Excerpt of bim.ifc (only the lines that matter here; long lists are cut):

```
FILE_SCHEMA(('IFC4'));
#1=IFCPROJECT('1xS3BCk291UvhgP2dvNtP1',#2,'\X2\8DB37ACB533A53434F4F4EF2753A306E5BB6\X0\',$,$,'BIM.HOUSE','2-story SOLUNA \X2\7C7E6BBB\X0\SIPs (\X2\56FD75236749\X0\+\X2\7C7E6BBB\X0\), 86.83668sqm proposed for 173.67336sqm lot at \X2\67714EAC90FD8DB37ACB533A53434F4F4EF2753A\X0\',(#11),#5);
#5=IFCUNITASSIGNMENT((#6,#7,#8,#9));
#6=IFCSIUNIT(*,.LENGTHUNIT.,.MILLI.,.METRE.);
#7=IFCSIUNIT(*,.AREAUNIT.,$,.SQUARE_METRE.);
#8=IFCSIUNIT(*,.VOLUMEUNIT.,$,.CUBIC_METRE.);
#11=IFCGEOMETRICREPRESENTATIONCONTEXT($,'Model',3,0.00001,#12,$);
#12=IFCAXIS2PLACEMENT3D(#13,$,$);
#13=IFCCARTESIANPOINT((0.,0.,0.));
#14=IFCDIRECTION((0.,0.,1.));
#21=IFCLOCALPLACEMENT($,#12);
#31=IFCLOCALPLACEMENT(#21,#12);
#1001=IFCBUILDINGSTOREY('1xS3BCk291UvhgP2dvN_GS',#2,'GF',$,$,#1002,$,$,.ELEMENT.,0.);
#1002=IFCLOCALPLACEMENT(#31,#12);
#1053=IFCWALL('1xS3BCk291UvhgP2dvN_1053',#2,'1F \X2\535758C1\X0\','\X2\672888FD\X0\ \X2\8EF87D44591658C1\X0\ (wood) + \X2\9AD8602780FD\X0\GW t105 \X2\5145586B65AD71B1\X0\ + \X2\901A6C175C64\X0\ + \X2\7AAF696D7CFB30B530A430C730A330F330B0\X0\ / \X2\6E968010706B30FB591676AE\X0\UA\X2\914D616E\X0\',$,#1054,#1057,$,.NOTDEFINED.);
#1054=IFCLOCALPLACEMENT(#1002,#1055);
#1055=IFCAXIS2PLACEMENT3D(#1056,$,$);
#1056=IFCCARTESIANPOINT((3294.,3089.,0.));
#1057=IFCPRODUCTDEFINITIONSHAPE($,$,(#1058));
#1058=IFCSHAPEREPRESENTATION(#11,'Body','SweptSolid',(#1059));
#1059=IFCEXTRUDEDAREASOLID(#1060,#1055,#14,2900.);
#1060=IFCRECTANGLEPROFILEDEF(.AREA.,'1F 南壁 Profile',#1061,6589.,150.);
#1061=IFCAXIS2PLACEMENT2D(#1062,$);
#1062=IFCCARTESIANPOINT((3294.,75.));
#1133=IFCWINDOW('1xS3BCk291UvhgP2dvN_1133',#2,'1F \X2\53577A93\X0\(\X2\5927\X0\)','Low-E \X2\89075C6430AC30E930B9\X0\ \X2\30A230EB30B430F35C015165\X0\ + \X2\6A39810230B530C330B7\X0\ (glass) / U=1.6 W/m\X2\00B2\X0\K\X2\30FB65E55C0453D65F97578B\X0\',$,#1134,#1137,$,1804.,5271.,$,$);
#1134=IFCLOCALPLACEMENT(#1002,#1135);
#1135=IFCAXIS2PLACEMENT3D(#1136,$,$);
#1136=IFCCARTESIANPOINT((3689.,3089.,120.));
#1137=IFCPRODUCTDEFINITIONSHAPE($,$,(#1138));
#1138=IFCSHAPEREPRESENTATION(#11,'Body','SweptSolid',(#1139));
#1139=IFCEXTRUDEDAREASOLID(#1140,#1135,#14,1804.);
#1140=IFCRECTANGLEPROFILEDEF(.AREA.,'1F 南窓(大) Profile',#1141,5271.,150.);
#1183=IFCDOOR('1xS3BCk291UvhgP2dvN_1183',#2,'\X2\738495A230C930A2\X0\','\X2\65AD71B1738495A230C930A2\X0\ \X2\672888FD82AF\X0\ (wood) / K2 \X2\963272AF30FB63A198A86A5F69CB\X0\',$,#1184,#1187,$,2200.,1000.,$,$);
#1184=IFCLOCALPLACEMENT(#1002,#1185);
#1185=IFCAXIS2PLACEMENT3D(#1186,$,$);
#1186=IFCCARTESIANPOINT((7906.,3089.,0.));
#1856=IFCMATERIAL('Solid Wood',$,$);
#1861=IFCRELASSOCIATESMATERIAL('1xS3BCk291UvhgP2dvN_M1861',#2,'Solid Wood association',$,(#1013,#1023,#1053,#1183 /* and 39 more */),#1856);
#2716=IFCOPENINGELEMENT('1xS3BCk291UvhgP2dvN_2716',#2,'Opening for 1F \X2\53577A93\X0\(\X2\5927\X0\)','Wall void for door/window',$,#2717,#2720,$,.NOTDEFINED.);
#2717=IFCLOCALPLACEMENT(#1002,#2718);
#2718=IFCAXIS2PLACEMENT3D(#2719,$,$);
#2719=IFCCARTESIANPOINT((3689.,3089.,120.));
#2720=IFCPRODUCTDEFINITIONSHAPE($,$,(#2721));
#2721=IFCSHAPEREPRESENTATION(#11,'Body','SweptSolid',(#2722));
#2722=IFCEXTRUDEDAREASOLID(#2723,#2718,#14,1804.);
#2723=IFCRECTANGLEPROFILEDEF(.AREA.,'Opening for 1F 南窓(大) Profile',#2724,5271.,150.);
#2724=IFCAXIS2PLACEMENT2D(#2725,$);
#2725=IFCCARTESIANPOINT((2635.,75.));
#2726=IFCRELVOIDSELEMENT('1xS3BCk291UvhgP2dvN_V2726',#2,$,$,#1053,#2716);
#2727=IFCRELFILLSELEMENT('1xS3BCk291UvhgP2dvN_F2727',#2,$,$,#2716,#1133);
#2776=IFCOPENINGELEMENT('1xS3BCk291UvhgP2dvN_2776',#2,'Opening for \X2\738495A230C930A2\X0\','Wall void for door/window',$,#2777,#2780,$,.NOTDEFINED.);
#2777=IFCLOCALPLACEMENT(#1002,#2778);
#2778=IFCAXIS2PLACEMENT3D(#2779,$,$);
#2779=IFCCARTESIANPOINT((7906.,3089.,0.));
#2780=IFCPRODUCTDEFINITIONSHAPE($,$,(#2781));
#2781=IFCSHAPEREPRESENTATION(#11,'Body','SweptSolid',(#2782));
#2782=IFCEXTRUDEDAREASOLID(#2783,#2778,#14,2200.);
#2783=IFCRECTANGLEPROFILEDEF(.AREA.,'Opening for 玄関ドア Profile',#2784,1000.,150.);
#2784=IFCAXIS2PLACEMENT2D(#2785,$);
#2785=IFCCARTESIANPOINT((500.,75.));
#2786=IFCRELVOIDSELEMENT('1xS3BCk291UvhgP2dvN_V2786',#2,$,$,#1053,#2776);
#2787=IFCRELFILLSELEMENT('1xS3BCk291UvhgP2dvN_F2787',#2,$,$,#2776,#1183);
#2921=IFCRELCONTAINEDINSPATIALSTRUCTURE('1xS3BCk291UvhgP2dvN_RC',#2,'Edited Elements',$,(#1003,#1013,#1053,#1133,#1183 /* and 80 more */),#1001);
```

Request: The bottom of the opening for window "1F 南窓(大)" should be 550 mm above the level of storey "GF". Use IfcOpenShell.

```python
import numpy as np
import ifcopenshell
import ifcopenshell.api.geometry
import ifcopenshell.geom
import ifcopenshell.util.element
import ifcopenshell.util.placement
import ifcopenshell.util.shape
import ifcopenshell.util.unit

model = ifcopenshell.open("bim.ifc")
unit_scale = ifcopenshell.util.unit.calculate_unit_scale(model)

window = model.by_id(1133)
opening = window.FillsVoids[0].RelatingOpeningElement
storey = ifcopenshell.util.element.get_container(window, ifc_class="IfcBuildingStorey")
level = ifcopenshell.util.placement.get_local_placement(storey.ObjectPlacement)[2, 3]

# The opening's origin need not be at the sill, so measure its lowest point.
shape = ifcopenshell.geom.create_shape(ifcopenshell.geom.settings(), opening)
bottom = ifcopenshell.util.shape.get_shape_bottom_elevation(shape, shape.geometry) / unit_scale
dz = level + 0.55 / unit_scale - bottom

shift = np.array([0.0, 0.0, dz])
# The window is not placed relative to its opening, so move both.
for product in (opening, window):
    matrix = ifcopenshell.util.placement.get_local_placement(product.ObjectPlacement)
    matrix[:3, 3] += shift
    ifcopenshell.api.geometry.edit_object_placement(model, product=product, matrix=matrix, is_si=False)

print(f"moved by {dz * unit_scale:+.3f} m")

model.write("bim_v2.ifc")
```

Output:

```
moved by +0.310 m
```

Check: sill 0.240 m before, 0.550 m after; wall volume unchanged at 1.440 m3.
